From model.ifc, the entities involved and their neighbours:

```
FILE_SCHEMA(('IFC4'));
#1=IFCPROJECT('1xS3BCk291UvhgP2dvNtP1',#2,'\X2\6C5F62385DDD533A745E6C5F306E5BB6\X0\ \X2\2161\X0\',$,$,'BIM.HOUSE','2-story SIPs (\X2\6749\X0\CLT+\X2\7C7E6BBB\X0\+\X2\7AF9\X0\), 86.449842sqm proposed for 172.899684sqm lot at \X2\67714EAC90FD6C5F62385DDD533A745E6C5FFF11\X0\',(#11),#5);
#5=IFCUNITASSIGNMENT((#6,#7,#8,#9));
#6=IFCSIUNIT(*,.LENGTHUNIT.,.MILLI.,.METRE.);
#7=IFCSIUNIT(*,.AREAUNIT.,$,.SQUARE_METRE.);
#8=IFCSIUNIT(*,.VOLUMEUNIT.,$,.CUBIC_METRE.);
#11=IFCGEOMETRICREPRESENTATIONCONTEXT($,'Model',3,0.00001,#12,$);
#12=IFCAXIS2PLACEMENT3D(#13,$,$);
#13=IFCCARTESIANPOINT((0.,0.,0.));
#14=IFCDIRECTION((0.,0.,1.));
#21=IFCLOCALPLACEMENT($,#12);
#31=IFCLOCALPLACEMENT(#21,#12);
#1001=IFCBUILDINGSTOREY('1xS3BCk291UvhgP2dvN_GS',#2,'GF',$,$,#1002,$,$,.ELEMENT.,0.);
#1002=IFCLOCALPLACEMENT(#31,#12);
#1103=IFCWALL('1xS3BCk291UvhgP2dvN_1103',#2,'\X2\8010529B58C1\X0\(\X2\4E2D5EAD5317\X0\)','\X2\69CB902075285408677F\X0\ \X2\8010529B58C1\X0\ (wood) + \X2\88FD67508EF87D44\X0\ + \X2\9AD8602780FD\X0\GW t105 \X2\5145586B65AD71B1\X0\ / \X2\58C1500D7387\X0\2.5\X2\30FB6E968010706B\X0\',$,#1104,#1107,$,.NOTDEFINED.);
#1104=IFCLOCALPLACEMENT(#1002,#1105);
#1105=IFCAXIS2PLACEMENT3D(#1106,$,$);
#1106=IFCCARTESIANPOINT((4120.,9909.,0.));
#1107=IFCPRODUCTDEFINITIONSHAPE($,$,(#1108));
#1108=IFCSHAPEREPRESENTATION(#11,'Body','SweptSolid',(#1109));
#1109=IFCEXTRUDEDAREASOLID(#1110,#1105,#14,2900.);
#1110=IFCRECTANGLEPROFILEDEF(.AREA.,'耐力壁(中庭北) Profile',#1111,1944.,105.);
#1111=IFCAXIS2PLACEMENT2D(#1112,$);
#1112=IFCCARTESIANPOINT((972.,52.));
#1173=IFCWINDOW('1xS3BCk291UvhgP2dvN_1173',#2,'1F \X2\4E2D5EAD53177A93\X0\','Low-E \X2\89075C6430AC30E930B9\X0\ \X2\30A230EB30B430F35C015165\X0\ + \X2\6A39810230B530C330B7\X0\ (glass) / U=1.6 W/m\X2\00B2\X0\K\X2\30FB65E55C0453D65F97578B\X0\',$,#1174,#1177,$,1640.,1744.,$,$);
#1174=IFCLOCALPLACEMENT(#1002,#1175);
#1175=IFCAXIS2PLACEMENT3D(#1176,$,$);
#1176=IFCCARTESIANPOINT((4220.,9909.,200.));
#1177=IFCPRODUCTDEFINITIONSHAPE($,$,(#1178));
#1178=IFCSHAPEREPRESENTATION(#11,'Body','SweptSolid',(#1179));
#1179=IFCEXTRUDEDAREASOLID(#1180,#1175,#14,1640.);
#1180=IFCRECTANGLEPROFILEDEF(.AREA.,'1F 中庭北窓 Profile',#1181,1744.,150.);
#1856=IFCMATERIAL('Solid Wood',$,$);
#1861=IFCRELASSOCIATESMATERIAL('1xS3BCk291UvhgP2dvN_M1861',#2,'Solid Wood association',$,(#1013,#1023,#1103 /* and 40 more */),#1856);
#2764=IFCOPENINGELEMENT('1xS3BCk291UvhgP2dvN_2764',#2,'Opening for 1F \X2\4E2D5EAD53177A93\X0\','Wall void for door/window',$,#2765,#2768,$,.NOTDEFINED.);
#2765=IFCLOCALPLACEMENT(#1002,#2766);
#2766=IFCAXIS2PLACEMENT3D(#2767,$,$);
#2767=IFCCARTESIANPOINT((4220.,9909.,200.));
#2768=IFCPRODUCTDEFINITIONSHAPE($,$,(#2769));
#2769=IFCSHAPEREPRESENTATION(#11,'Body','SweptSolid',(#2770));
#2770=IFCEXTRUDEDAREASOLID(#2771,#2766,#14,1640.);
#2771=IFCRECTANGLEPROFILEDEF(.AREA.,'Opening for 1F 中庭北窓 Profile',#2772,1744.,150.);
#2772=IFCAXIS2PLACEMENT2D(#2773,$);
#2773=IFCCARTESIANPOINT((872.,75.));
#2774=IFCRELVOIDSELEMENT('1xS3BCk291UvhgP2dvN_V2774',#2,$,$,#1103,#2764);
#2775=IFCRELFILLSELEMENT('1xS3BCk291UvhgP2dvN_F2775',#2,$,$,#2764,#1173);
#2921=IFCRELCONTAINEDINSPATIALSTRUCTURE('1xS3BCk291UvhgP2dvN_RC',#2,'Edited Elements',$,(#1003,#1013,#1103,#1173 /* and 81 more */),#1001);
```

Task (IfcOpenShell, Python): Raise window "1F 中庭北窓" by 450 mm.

```python
import numpy as np
import ifcopenshell
import ifcopenshell.api.geometry
import ifcopenshell.util.placement
import ifcopenshell.util.unit

model = ifcopenshell.open("model.ifc")
unit_scale = ifcopenshell.util.unit.calculate_unit_scale(model)

window = model.by_id(1173)
opening = window.FillsVoids[0].RelatingOpeningElement
dz = 0.45 / unit_scale

shift = np.array([0.0, 0.0, dz])
# The window is not placed relative to its opening, so move both.
for product in (opening, window):
    matrix = ifcopenshell.util.placement.get_local_placement(product.ObjectPlacement)
    matrix[:3, 3] += shift
    ifcopenshell.api.geometry.edit_object_placement(model, product=product, matrix=matrix, is_si=False)

print(f"moved by {dz * unit_scale:+.3f} m")

model.write("model_edited.ifc")
```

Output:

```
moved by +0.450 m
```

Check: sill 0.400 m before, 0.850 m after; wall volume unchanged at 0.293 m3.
